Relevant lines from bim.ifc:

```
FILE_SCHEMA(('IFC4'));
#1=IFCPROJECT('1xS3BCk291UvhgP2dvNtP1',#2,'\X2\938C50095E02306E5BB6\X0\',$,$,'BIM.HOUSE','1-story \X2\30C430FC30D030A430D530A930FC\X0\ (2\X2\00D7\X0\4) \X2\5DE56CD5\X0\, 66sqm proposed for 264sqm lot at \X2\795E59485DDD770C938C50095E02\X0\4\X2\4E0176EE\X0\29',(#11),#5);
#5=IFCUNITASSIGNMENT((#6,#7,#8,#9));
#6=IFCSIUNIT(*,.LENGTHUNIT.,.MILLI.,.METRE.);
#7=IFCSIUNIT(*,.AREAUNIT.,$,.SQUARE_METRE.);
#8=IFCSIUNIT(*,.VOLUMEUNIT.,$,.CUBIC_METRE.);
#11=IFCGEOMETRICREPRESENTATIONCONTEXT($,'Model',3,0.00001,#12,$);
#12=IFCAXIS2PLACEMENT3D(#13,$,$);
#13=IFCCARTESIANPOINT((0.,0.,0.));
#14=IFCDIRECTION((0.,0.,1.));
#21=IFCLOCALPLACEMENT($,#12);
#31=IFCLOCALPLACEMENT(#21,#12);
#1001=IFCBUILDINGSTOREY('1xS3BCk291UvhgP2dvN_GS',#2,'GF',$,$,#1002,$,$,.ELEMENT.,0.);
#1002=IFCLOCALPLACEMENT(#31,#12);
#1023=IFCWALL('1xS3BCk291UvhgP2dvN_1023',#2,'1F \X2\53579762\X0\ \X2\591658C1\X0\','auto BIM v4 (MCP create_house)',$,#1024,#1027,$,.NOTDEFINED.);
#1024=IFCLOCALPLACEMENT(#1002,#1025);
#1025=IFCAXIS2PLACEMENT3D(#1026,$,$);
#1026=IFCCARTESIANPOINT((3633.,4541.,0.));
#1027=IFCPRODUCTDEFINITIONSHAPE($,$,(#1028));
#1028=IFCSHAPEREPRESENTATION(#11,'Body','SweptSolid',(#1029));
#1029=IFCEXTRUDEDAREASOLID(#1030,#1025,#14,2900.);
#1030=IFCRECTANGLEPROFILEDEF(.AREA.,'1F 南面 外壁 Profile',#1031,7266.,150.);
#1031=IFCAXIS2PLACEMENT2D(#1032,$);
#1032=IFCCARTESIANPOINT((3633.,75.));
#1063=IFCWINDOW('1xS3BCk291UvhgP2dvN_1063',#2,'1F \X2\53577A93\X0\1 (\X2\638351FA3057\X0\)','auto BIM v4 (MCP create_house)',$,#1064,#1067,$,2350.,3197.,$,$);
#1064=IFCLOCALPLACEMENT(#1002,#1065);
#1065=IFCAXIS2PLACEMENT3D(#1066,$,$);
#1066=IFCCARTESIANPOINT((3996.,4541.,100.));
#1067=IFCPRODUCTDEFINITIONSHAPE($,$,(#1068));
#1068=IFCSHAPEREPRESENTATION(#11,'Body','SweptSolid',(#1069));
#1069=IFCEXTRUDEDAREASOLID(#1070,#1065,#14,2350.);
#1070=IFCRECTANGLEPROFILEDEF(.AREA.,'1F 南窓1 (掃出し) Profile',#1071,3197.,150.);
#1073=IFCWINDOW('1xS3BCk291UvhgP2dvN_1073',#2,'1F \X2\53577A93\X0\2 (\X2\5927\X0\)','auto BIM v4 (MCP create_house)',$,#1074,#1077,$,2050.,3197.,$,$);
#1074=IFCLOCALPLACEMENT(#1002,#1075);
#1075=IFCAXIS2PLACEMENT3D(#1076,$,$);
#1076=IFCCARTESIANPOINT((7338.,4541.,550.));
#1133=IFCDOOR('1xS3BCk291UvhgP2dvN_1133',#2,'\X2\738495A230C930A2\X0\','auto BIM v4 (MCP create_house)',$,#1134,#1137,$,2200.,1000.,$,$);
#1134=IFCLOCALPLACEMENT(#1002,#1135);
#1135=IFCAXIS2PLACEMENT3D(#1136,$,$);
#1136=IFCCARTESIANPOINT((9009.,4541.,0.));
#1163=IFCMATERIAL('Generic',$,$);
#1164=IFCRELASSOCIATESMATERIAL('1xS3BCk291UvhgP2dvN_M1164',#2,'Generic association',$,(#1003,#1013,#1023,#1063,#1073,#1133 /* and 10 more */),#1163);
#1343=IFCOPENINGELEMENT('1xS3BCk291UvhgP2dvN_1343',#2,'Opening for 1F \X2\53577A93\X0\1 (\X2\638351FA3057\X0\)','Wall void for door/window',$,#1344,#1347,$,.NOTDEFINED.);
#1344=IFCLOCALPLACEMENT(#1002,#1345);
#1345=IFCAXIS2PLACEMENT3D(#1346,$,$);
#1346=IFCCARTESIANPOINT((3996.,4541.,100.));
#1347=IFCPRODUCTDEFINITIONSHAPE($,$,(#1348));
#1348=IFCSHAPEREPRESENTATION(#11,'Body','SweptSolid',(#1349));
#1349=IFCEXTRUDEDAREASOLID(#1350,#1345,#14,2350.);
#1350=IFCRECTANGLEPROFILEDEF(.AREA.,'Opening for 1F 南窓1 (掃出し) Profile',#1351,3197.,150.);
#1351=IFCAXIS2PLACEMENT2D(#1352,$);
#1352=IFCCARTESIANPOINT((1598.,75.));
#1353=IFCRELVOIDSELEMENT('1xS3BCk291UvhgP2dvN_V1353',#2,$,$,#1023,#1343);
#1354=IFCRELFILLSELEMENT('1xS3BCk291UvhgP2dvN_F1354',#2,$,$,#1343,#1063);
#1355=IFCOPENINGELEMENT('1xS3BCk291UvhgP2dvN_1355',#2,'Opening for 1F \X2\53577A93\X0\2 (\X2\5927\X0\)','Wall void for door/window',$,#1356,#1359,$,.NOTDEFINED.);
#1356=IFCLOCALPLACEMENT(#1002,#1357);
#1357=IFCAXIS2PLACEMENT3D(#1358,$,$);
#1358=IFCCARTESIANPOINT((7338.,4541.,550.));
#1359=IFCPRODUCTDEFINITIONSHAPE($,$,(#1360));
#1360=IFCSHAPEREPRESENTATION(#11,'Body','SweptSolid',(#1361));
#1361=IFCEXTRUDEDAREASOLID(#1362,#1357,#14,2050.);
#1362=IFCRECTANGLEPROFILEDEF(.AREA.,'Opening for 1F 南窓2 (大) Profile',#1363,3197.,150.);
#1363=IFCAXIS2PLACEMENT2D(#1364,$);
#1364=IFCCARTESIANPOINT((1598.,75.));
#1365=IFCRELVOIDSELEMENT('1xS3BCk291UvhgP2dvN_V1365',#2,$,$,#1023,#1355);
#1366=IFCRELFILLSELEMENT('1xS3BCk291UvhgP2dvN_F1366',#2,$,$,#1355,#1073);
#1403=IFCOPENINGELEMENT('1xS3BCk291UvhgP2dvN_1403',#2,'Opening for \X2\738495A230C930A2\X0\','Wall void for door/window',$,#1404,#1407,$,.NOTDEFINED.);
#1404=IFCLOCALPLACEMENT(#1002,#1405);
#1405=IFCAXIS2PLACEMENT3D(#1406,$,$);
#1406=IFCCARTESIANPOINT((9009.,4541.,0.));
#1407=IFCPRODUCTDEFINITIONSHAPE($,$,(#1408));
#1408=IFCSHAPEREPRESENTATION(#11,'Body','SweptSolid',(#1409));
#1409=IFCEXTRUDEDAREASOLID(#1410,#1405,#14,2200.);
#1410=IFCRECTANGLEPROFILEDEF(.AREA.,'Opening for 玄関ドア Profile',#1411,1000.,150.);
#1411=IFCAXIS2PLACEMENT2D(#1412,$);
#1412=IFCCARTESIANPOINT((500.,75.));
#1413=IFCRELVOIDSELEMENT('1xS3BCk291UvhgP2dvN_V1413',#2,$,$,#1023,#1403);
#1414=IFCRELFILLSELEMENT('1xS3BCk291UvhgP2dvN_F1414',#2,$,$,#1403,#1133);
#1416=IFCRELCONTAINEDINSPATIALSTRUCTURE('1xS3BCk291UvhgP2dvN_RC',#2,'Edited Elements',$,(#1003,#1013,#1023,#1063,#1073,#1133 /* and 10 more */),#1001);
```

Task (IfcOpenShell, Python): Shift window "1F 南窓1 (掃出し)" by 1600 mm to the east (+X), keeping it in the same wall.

```python
import ifcopenshell
import ifcopenshell.api.geometry
import ifcopenshell.util.placement

model = ifcopenshell.open("bim.ifc")

window = model.by_guid("1xS3BCk291UvhgP2dvN_1063")
opening = window.FillsVoids[0].RelatingOpeningElement
wall = opening.VoidsElements[0].RelatingBuildingElement

wall_matrix = ifcopenshell.util.placement.get_local_placement(wall.ObjectPlacement)
shift = wall_matrix[:3, 0] * 1600.0
before = ifcopenshell.util.placement.get_local_placement(window.ObjectPlacement)[:3, 3].copy()

# The window is not placed relative to its opening, so move both.
for product in (opening, window):
    matrix = ifcopenshell.util.placement.get_local_placement(product.ObjectPlacement)
    matrix[:3, 3] += shift
    ifcopenshell.api.geometry.edit_object_placement(model, product=product, matrix=matrix, is_si=False)

after = ifcopenshell.util.placement.get_local_placement(window.ObjectPlacement)[:3, 3]
print("window moved by", (after - before).round(3) + 0.0)

model.write("bim_edited.ifc")
```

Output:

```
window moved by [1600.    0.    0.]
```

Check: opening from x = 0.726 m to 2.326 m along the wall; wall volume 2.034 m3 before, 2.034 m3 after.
